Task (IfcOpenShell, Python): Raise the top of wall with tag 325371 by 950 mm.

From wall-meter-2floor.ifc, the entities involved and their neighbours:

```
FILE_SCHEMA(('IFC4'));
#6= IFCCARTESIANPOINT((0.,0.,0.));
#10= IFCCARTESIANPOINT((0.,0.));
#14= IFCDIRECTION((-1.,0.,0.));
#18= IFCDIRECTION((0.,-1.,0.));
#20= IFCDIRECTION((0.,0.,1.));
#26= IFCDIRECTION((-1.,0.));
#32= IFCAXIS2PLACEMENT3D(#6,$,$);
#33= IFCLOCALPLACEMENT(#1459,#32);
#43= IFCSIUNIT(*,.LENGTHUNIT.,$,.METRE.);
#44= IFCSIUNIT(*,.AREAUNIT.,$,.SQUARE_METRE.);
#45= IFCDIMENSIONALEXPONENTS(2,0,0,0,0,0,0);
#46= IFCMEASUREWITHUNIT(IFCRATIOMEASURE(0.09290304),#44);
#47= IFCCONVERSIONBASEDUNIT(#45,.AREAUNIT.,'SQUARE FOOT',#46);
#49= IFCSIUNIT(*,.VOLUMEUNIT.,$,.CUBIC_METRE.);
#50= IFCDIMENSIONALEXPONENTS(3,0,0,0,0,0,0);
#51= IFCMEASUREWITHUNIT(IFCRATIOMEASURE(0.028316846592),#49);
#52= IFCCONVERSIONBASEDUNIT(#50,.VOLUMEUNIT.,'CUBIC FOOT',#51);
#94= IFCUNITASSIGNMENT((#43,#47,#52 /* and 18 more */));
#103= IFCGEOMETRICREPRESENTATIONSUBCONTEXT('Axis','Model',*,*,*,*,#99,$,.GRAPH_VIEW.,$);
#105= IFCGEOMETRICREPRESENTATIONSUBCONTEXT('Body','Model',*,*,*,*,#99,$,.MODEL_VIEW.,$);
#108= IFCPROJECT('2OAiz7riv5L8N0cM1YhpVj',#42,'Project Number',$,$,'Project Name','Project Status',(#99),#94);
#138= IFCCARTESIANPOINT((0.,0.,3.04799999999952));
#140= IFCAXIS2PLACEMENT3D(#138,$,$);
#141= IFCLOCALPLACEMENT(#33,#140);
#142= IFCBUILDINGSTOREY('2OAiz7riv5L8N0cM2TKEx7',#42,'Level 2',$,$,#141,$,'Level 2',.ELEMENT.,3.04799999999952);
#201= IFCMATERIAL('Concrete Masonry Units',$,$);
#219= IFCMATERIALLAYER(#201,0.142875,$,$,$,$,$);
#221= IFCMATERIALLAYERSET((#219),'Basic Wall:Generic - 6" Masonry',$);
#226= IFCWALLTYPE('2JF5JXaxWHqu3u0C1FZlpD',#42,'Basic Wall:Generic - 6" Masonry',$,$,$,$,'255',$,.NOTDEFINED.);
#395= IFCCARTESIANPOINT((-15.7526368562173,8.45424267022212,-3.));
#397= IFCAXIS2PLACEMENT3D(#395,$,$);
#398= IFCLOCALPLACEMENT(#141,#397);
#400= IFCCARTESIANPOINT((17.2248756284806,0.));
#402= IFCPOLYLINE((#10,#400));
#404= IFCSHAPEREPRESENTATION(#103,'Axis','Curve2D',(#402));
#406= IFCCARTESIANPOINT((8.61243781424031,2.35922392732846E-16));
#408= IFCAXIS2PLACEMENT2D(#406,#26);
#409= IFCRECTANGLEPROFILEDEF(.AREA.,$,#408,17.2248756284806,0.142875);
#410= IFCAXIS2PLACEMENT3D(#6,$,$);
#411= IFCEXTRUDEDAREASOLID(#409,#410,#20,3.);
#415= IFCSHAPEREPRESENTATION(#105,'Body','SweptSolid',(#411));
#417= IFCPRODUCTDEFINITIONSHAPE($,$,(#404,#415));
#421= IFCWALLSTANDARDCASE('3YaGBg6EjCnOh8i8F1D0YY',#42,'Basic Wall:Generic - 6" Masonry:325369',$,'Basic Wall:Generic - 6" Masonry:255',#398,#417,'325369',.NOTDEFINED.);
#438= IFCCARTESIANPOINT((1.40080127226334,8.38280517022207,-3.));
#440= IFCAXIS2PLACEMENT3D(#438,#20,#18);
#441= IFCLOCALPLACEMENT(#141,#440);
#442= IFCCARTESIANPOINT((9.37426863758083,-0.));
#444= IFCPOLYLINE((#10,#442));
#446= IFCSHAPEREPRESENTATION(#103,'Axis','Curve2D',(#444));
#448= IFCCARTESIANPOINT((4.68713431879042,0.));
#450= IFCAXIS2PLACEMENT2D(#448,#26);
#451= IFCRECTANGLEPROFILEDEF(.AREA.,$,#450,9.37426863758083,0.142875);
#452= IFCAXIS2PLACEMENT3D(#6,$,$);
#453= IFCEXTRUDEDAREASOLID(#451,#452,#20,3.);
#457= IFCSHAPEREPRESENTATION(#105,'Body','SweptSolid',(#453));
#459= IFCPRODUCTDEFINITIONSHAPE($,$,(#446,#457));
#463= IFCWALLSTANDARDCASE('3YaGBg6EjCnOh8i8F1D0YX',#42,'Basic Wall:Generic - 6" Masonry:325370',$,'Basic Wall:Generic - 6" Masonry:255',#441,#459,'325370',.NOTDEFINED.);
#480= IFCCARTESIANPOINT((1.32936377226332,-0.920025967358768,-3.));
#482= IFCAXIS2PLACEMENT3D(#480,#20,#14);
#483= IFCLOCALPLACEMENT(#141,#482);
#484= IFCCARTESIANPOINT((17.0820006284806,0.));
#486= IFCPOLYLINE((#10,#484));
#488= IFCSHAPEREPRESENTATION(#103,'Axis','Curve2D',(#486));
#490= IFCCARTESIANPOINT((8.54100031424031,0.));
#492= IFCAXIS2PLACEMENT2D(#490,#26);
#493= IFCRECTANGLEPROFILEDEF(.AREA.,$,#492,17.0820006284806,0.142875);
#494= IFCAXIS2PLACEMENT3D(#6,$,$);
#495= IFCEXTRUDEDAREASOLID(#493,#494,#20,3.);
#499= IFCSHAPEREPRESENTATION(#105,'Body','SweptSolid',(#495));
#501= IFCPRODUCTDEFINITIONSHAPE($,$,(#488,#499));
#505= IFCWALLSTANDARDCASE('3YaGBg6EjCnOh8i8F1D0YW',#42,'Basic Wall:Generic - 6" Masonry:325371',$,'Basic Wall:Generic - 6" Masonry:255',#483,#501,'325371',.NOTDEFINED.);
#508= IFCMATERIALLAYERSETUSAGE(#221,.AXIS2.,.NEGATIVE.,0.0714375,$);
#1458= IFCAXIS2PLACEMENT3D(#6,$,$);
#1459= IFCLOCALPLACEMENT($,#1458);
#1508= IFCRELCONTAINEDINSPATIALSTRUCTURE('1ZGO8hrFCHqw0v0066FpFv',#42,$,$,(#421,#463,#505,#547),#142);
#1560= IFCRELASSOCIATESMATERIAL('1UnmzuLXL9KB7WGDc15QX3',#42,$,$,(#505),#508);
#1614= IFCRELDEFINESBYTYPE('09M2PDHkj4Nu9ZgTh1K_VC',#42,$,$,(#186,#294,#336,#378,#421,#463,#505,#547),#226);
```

```python
import ifcopenshell
import ifcopenshell.geom
import ifcopenshell.util.representation
import ifcopenshell.util.shape
import ifcopenshell.util.unit

model = ifcopenshell.open("wall-meter-2floor.ifc")
unit_scale = ifcopenshell.util.unit.calculate_unit_scale(model)
settings = ifcopenshell.geom.settings()


def volume(element):
    """Net volume in cubic metres, openings subtracted."""
    shape = ifcopenshell.geom.create_shape(settings, element)
    return ifcopenshell.util.shape.get_volume(shape.geometry)


wall = model.by_guid("3YaGBg6EjCnOh8i8F1D0YW")
before = volume(wall)

body = ifcopenshell.util.representation.get_representation(wall, "Model", "Body")
solid = body.Items[0]
old_height = solid.Depth
solid.Depth += 0.95 / unit_scale
after = volume(wall)

print(f"height {old_height:g} -> {solid.Depth:g}, volume {before:.3f} -> {after:.3f} m3")

model.write("wall-meter-2floor_updated.ifc")
```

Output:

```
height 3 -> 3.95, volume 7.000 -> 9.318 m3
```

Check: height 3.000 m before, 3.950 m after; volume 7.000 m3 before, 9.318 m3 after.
